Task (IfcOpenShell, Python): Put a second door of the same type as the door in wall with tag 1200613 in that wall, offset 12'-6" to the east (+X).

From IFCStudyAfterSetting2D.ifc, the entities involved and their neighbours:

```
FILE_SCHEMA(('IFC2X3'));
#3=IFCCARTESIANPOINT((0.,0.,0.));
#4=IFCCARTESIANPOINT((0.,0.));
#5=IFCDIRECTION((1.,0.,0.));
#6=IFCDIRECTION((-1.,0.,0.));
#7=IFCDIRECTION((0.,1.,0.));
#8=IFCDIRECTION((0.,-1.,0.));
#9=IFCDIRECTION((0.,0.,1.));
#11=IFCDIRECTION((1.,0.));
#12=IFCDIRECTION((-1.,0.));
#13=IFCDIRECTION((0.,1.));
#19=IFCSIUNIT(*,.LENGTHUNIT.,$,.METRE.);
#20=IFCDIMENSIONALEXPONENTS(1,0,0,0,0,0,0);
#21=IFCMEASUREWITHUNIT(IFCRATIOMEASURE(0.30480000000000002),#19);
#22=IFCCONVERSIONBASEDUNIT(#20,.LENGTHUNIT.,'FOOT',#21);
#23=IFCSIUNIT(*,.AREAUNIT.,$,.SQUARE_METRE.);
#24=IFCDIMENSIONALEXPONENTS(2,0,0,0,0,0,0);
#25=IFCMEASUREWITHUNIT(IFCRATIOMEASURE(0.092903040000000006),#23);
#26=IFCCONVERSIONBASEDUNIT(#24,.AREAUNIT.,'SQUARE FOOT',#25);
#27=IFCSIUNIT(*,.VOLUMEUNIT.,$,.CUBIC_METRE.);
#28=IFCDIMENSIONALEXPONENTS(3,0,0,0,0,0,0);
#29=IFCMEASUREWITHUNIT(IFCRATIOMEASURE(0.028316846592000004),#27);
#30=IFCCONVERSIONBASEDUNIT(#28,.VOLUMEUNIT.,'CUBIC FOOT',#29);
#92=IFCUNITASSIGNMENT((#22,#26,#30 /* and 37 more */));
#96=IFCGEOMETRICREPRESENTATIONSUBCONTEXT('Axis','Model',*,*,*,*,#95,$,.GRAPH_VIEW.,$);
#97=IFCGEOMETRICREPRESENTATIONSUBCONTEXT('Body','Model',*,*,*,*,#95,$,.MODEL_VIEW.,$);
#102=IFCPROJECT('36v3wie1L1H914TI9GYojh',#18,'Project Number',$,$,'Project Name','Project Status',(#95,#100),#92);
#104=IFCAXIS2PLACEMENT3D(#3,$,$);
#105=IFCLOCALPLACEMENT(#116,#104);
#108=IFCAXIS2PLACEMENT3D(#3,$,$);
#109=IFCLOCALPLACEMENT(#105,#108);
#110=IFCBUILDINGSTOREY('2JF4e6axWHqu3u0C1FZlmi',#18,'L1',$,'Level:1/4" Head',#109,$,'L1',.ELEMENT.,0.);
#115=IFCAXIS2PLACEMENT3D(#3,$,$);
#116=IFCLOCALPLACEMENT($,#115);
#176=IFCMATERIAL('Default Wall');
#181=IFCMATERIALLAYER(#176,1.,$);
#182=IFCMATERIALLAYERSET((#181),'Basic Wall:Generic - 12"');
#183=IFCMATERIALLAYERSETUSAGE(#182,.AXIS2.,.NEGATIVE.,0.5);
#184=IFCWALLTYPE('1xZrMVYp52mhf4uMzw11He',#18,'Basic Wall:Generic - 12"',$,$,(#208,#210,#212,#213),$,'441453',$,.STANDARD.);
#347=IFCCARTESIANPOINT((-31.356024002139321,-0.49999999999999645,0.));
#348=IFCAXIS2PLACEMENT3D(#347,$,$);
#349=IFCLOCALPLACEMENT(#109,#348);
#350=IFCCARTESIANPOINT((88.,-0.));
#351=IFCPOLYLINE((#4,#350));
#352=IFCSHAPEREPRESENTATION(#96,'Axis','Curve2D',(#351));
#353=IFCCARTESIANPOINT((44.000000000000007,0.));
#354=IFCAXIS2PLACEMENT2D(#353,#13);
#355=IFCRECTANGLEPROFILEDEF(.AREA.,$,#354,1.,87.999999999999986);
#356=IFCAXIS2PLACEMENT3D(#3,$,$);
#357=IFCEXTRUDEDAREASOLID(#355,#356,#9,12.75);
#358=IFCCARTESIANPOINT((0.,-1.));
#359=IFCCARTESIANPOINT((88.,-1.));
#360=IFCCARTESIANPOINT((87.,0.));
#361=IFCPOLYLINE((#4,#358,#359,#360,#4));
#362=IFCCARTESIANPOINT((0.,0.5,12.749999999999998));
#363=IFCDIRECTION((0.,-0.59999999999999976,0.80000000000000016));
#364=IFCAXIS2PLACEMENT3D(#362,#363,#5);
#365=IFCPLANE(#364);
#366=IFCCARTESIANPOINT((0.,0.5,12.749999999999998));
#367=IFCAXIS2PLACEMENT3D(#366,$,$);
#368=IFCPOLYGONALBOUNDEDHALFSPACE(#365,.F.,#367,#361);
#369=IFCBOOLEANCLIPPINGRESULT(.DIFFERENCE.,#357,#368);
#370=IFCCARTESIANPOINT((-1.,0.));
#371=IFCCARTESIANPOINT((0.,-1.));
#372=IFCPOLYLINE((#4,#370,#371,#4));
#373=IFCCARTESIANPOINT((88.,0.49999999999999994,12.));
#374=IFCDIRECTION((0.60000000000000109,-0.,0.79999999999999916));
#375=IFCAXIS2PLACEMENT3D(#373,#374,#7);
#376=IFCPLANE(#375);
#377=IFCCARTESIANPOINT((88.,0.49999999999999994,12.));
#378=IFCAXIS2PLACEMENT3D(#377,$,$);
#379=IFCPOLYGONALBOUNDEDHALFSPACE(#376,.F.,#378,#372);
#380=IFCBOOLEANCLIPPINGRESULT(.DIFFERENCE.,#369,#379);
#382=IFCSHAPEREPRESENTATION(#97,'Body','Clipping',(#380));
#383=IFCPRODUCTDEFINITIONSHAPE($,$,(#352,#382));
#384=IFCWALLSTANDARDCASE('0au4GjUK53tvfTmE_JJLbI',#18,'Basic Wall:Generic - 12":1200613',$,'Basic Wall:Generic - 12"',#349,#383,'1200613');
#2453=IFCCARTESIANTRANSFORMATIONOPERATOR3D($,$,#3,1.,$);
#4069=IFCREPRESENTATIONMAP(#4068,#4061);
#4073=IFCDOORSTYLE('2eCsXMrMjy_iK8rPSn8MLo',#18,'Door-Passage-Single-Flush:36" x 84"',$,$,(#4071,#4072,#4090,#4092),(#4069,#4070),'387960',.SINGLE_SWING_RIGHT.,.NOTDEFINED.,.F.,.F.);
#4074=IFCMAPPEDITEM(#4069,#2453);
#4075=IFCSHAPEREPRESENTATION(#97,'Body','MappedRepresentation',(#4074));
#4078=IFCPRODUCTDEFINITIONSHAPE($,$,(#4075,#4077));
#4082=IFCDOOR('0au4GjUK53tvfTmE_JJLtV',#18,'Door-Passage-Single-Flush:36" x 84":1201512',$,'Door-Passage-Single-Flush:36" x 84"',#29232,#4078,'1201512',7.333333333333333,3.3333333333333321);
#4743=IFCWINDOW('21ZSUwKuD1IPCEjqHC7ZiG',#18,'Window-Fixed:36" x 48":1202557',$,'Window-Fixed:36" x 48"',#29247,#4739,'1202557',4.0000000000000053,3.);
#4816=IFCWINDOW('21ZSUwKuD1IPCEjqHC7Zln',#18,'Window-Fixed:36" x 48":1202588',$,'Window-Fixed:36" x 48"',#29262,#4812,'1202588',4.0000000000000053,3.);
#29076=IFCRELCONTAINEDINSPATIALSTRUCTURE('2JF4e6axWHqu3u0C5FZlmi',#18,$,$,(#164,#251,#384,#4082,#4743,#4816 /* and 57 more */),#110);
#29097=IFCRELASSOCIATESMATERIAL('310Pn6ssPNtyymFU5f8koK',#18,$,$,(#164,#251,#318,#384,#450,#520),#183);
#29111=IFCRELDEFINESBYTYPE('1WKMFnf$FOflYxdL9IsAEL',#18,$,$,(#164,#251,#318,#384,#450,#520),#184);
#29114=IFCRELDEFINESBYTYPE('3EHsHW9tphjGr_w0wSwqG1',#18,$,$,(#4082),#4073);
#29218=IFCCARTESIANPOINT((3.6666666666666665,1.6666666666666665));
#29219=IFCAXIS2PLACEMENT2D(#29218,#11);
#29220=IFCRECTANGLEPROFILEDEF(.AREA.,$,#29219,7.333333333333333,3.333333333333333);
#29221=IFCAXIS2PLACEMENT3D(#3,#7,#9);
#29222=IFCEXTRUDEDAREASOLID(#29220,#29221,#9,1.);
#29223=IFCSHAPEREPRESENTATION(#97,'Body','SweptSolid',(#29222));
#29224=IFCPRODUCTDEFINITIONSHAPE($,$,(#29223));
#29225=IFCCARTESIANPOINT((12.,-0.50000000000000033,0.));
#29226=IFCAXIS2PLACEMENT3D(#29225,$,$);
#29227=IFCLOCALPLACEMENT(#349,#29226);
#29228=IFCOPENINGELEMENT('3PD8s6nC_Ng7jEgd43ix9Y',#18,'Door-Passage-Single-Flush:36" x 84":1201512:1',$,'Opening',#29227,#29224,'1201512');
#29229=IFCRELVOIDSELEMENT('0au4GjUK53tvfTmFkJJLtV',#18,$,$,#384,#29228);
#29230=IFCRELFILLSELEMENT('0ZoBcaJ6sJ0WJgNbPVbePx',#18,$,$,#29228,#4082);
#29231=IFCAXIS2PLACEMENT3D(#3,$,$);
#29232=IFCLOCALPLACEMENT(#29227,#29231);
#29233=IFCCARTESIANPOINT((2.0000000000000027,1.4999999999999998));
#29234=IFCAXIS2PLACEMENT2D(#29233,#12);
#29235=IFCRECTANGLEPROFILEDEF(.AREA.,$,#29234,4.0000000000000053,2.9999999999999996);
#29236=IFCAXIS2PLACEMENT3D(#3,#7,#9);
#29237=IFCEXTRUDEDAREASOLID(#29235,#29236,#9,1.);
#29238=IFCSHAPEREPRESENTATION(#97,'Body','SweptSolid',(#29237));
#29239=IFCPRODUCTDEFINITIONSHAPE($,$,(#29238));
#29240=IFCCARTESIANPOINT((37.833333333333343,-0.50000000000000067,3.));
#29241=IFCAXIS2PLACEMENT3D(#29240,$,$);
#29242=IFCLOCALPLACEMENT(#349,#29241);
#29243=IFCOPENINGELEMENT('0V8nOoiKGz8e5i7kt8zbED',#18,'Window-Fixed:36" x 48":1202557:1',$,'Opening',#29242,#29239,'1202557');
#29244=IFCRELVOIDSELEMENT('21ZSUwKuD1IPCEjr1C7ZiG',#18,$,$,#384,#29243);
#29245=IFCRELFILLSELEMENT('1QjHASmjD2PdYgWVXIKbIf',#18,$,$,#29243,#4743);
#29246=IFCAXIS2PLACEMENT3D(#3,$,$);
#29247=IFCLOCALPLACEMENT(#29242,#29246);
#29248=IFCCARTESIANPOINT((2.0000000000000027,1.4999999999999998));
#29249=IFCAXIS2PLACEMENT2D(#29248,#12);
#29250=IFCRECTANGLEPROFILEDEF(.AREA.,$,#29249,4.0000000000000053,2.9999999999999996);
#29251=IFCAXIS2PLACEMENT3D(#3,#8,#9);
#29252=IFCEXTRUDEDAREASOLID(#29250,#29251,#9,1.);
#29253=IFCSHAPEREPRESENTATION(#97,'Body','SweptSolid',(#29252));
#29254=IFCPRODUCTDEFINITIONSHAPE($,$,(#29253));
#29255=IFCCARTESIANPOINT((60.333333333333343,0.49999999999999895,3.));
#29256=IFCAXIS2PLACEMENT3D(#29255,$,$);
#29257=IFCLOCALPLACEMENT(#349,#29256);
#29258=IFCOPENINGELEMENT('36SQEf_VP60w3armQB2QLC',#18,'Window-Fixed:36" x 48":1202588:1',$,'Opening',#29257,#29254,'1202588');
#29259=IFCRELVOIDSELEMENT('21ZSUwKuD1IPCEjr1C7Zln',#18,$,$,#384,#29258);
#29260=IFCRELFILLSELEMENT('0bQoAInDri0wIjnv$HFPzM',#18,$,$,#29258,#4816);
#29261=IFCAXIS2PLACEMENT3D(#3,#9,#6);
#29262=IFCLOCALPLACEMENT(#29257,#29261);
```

```python
import ifcopenshell
import ifcopenshell.api.feature
import ifcopenshell.api.geometry
import ifcopenshell.api.root
import ifcopenshell.geom
import ifcopenshell.util.element
import ifcopenshell.util.placement
import ifcopenshell.util.shape
import ifcopenshell.util.unit

model = ifcopenshell.open("IFCStudyAfterSetting2D.ifc")
unit_scale = ifcopenshell.util.unit.calculate_unit_scale(model)
settings = ifcopenshell.geom.settings()


def volume(element):
    """Net volume in cubic metres, openings subtracted."""
    shape = ifcopenshell.geom.create_shape(settings, element)
    return ifcopenshell.util.shape.get_volume(shape.geometry)


def reuse_history(source, copy):
    """copy_class also copies each property set's owner history, people and application; keep the originals."""
    for rel in copy.IsDefinedBy:
        if rel.is_a("IfcRelDefinesByProperties") and (history := rel.RelatingPropertyDefinition.OwnerHistory):
            rel.RelatingPropertyDefinition.OwnerHistory = source.OwnerHistory
            ifcopenshell.util.element.remove_deep2(model, history)


door = model.by_id(4082)
opening = door.FillsVoids[0].RelatingOpeningElement
wall = opening.VoidsElements[0].RelatingBuildingElement
before = volume(wall)
shift = ifcopenshell.util.placement.get_local_placement(wall.ObjectPlacement)[:3, 0] * 150 * 0.0254 / unit_scale

# copy_class copies the void relationship, type, container and properties, but no geometry.
new_opening = ifcopenshell.api.root.copy_class(model, product=opening)
new_opening.Representation = ifcopenshell.util.element.copy_deep(
    model, opening.Representation, exclude=["IfcGeometricRepresentationContext", "IfcRepresentationMap"]
)
new_opening.Name = 'Door-Passage-Single-Flush:36" x 84"'
new_opening.Tag = None
new_door = ifcopenshell.api.root.copy_class(model, product=door)
new_door.Representation = ifcopenshell.util.element.copy_deep(
    model, door.Representation, exclude=["IfcGeometricRepresentationContext", "IfcRepresentationMap"]
)
new_door.Name = 'Door-Passage-Single-Flush:36" x 84"'
new_door.Tag = None
reuse_history(door, new_door)
fills = ifcopenshell.api.feature.add_filling(model, opening=new_opening, element=new_door)
fills.OwnerHistory = new_door.OwnerHistory  # required in IFC2X3

for old, new in ((opening, new_opening), (door, new_door)):
    matrix = ifcopenshell.util.placement.get_local_placement(old.ObjectPlacement)
    matrix[:3, 3] += shift
    ifcopenshell.api.geometry.edit_object_placement(model, product=new, matrix=matrix, is_si=False)

after = volume(wall)

print(f"wall volume {before:.3f} -> {after:.3f} m3")

model.write("IFCStudyAfterSetting2D_rev.ifc")
```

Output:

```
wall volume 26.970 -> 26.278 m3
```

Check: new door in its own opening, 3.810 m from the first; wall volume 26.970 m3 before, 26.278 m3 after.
